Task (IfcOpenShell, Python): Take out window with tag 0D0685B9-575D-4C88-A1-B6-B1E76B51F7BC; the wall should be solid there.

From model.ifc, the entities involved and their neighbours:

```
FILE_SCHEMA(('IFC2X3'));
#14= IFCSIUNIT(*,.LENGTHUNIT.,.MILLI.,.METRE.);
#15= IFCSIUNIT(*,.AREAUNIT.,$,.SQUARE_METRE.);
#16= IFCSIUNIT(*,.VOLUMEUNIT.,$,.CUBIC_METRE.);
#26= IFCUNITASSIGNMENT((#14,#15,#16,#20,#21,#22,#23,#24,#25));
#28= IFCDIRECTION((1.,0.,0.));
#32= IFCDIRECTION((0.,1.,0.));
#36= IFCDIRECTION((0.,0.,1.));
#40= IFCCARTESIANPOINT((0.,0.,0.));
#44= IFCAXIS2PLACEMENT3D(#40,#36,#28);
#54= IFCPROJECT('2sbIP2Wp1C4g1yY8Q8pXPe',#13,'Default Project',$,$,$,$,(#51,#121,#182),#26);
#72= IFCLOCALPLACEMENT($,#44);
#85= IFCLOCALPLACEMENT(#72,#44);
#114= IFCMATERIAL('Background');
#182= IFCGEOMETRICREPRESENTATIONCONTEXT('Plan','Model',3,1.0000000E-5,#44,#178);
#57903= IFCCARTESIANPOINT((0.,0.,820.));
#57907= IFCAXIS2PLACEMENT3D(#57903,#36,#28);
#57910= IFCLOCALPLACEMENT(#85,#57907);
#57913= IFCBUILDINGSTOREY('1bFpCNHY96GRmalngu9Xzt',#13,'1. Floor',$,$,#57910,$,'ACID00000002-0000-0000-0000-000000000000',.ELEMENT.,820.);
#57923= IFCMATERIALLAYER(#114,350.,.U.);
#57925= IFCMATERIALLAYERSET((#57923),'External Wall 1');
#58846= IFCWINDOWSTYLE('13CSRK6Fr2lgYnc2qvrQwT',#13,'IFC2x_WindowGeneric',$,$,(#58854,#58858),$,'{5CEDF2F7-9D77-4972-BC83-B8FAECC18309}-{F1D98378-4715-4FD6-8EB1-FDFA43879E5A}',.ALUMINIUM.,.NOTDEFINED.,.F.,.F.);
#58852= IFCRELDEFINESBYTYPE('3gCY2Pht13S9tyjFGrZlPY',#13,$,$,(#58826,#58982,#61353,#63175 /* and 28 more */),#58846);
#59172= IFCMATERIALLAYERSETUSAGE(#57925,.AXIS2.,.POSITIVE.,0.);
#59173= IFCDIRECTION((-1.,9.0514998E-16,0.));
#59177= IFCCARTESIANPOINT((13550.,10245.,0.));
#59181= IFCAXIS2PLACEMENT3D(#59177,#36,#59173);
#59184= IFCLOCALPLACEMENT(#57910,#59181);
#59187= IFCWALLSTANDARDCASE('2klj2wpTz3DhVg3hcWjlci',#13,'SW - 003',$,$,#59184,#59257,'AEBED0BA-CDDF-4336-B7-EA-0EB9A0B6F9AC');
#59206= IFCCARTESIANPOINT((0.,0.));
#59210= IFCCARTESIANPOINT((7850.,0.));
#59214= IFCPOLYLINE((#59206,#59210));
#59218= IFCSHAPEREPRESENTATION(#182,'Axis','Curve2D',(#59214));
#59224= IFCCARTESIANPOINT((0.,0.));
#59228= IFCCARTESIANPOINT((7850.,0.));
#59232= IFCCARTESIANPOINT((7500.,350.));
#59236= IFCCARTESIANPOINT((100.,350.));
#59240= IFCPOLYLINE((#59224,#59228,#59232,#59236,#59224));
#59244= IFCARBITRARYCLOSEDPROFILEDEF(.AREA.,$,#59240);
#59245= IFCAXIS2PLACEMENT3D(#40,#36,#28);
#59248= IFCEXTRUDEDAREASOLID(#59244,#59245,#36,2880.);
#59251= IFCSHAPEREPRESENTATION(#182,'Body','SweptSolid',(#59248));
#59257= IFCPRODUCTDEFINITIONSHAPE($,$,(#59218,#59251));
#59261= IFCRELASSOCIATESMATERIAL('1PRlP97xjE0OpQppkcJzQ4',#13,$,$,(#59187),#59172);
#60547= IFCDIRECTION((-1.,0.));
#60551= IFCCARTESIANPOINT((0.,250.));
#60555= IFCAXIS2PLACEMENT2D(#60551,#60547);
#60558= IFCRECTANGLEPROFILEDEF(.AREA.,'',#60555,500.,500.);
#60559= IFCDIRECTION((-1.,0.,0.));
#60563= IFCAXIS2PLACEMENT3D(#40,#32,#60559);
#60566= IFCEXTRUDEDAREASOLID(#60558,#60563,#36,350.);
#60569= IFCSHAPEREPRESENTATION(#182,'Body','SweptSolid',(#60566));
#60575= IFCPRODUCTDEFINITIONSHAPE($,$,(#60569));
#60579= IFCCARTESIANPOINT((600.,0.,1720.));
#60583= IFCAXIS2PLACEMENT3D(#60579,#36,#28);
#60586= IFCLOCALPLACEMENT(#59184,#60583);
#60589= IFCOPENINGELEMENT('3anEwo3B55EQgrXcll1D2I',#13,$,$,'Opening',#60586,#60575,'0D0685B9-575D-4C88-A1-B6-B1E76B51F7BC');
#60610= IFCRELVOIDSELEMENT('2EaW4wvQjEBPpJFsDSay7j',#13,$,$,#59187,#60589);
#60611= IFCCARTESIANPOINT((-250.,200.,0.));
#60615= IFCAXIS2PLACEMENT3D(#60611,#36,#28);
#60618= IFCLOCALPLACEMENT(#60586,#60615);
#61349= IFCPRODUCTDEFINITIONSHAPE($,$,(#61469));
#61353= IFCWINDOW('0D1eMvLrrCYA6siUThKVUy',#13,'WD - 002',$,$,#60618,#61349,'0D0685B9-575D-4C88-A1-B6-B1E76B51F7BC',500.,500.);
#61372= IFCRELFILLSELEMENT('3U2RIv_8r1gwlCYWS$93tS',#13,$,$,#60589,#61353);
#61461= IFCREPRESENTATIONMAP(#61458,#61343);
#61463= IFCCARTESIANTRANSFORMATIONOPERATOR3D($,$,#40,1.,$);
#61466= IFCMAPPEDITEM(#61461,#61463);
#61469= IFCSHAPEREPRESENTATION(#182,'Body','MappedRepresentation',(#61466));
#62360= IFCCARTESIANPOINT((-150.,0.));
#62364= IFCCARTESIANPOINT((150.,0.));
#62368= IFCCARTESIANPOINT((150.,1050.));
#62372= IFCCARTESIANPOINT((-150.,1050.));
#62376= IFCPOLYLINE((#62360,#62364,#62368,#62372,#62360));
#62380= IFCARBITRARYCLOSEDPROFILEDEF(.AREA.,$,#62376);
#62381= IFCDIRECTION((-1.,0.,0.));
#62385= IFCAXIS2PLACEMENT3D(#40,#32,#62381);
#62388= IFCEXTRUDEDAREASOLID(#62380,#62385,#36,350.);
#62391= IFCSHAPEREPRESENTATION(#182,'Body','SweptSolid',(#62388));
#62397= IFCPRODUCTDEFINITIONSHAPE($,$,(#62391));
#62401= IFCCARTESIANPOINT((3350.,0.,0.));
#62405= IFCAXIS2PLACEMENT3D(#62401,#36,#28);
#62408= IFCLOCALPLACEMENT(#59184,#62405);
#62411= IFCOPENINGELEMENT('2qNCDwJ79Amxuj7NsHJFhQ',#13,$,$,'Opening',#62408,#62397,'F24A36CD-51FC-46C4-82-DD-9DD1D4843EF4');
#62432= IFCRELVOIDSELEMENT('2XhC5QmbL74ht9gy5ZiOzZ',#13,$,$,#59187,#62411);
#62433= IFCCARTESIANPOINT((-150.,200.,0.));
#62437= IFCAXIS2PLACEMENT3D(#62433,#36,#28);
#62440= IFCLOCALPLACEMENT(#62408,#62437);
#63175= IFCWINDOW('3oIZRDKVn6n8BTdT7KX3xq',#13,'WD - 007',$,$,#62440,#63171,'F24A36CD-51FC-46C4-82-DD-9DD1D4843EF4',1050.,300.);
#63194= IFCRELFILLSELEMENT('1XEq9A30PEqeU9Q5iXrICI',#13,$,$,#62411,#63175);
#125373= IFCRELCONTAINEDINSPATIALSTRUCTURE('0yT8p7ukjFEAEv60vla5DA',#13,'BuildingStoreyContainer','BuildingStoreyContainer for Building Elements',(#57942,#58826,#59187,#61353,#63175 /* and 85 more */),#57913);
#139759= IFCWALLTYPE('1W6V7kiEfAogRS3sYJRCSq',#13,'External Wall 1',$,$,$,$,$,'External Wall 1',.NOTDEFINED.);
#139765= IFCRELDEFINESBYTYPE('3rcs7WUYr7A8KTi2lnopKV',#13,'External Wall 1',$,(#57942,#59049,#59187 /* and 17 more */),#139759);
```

```python
import ifcopenshell
import ifcopenshell.api.feature
import ifcopenshell.api.root
import ifcopenshell.geom
import ifcopenshell.util.shape

model = ifcopenshell.open("model.ifc")
settings = ifcopenshell.geom.settings()


def volume(element):
    """Net volume in cubic metres, openings subtracted."""
    shape = ifcopenshell.geom.create_shape(settings, element)
    return ifcopenshell.util.shape.get_volume(shape.geometry)


window = model.by_guid("0D1eMvLrrCYA6siUThKVUy")
opening = window.FillsVoids[0].RelatingOpeningElement
wall = opening.VoidsElements[0].RelatingBuildingElement
before = volume(wall)

ifcopenshell.api.root.remove_product(model, product=window)
ifcopenshell.api.feature.remove_feature(model, feature=opening)

after = volume(wall)

print(f"wall volume {before:.3f} -> {after:.3f} m3")

model.write("model-out.ifc")
```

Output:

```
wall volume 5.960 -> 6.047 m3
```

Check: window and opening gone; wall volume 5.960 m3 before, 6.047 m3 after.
